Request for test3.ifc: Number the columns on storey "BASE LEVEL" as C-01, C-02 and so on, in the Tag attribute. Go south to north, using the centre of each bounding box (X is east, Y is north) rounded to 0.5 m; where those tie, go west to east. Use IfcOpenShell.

First a look at what the model holds.

```python
import ifcopenshell
import ifcopenshell.util.element
import ifcopenshell.util.placement

model = ifcopenshell.open("test3.ifc")
print(model.schema)
storey = next(s for s in model.by_type("IfcBuildingStorey") if s.Name == "BASE LEVEL")
columns = [e for e in ifcopenshell.util.element.get_decomposition(storey) if e.is_a("IfcColumn")]
for e in sorted(columns, key=lambda e: e.id()):
    origin = ifcopenshell.util.placement.get_local_placement(e.ObjectPlacement)[:3, 3]
    print(e.id(), e.Tag, e.Name, origin.round(2) + 0.0, sep=" | ")
```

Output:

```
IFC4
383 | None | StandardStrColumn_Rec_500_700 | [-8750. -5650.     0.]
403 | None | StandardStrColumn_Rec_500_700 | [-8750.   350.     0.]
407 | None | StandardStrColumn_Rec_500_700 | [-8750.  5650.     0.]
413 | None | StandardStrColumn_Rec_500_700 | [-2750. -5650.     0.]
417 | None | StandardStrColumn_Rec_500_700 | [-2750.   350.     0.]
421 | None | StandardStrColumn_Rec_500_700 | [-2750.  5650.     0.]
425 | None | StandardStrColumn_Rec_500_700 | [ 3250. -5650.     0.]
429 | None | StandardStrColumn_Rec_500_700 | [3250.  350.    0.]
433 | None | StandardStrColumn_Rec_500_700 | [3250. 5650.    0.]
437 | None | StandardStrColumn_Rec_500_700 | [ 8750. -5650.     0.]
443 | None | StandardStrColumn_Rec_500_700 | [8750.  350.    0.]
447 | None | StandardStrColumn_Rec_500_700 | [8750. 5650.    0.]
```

```python
import ifcopenshell
import ifcopenshell.geom
import ifcopenshell.util.element
import ifcopenshell.util.shape

model = ifcopenshell.open("test3.ifc")
settings = ifcopenshell.geom.settings()
settings.set("use-world-coords", True)


def centre(element):
    shape = ifcopenshell.geom.create_shape(settings, element)
    return ifcopenshell.util.shape.get_bbox_centroid(shape.geometry)


storey = next(s for s in model.by_type("IfcBuildingStorey") if s.Name == "BASE LEVEL")
columns = [e for e in ifcopenshell.util.element.get_decomposition(storey) if e.is_a("IfcColumn")]

# Insertion points can sit at a corner or the storey origin, so sort by the geometry (in metres).
centres = {e: centre(e) for e in columns}
columns.sort(key=lambda e: (round(centres[e][1] / 0.5), centres[e][0]))

for i, e in enumerate(columns, start=1):
    number = f"C-{i:02d}"
    e.Tag = number
    print(e.id(), number)

model.write("test3_rev.ifc")
```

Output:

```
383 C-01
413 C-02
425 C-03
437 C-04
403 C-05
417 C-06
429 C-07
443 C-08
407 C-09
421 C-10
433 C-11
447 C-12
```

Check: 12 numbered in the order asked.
